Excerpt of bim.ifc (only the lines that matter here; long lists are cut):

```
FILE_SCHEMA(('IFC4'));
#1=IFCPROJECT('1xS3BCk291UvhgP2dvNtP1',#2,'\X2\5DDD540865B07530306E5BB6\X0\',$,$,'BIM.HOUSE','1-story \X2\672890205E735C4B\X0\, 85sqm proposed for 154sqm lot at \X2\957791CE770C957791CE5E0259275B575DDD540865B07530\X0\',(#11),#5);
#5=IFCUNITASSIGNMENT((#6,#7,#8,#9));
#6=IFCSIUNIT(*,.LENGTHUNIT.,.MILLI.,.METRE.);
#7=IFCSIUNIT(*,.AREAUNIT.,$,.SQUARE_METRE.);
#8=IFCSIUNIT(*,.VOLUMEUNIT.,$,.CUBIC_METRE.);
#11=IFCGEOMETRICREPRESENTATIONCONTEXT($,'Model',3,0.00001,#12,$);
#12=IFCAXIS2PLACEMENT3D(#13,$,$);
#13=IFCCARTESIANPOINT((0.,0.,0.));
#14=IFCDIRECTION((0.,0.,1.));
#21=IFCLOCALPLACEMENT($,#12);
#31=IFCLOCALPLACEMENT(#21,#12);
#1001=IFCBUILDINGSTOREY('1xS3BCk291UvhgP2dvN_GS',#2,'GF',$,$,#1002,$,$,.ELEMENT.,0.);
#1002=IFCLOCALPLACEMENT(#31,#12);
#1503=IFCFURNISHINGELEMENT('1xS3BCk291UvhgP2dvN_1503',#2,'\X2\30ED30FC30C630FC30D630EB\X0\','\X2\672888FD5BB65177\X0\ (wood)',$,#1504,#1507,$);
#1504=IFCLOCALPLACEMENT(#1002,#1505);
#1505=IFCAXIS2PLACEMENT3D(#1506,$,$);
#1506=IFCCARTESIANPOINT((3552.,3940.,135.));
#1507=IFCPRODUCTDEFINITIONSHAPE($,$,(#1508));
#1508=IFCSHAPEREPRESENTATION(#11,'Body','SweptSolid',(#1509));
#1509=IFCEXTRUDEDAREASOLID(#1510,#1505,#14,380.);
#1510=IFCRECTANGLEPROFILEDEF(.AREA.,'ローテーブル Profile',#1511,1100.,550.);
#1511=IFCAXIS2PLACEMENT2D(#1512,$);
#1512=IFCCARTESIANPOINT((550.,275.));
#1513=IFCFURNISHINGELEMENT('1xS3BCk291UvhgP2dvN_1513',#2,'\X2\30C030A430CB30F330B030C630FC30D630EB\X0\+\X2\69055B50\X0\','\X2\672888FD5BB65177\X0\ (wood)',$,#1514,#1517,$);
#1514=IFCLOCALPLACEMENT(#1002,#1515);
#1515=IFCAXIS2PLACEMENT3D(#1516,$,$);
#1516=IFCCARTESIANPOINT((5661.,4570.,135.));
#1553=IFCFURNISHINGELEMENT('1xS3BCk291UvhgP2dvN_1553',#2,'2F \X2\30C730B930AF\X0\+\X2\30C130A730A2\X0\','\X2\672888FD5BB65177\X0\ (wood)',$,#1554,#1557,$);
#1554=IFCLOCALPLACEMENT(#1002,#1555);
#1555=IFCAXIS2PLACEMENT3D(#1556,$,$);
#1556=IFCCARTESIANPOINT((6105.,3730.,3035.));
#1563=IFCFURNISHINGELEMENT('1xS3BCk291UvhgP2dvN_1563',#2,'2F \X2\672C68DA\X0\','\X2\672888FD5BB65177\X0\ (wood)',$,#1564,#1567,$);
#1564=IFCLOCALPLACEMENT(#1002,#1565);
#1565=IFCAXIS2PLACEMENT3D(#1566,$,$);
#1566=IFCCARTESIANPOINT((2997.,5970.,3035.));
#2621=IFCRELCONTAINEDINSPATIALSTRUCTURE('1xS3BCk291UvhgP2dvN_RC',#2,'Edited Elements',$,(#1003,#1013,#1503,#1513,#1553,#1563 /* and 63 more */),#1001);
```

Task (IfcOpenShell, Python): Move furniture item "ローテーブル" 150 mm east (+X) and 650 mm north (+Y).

```python
import ifcopenshell
import ifcopenshell.api.geometry
import ifcopenshell.util.placement

model = ifcopenshell.open("bim.ifc")

item = model.by_guid("1xS3BCk291UvhgP2dvN_1503")
matrix = ifcopenshell.util.placement.get_local_placement(item.ObjectPlacement)
matrix[0, 3] += 150.0
matrix[1, 3] += 650.0
ifcopenshell.api.geometry.edit_object_placement(model, product=item, matrix=matrix, is_si=False)

print(ifcopenshell.util.placement.get_local_placement(item.ObjectPlacement).round(3) + 0.0)

model.write("bim_rev.ifc")
```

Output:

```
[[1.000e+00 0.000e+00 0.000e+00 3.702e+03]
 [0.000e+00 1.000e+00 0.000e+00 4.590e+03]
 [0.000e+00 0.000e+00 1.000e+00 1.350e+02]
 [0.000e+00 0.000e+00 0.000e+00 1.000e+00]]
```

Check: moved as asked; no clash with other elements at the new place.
